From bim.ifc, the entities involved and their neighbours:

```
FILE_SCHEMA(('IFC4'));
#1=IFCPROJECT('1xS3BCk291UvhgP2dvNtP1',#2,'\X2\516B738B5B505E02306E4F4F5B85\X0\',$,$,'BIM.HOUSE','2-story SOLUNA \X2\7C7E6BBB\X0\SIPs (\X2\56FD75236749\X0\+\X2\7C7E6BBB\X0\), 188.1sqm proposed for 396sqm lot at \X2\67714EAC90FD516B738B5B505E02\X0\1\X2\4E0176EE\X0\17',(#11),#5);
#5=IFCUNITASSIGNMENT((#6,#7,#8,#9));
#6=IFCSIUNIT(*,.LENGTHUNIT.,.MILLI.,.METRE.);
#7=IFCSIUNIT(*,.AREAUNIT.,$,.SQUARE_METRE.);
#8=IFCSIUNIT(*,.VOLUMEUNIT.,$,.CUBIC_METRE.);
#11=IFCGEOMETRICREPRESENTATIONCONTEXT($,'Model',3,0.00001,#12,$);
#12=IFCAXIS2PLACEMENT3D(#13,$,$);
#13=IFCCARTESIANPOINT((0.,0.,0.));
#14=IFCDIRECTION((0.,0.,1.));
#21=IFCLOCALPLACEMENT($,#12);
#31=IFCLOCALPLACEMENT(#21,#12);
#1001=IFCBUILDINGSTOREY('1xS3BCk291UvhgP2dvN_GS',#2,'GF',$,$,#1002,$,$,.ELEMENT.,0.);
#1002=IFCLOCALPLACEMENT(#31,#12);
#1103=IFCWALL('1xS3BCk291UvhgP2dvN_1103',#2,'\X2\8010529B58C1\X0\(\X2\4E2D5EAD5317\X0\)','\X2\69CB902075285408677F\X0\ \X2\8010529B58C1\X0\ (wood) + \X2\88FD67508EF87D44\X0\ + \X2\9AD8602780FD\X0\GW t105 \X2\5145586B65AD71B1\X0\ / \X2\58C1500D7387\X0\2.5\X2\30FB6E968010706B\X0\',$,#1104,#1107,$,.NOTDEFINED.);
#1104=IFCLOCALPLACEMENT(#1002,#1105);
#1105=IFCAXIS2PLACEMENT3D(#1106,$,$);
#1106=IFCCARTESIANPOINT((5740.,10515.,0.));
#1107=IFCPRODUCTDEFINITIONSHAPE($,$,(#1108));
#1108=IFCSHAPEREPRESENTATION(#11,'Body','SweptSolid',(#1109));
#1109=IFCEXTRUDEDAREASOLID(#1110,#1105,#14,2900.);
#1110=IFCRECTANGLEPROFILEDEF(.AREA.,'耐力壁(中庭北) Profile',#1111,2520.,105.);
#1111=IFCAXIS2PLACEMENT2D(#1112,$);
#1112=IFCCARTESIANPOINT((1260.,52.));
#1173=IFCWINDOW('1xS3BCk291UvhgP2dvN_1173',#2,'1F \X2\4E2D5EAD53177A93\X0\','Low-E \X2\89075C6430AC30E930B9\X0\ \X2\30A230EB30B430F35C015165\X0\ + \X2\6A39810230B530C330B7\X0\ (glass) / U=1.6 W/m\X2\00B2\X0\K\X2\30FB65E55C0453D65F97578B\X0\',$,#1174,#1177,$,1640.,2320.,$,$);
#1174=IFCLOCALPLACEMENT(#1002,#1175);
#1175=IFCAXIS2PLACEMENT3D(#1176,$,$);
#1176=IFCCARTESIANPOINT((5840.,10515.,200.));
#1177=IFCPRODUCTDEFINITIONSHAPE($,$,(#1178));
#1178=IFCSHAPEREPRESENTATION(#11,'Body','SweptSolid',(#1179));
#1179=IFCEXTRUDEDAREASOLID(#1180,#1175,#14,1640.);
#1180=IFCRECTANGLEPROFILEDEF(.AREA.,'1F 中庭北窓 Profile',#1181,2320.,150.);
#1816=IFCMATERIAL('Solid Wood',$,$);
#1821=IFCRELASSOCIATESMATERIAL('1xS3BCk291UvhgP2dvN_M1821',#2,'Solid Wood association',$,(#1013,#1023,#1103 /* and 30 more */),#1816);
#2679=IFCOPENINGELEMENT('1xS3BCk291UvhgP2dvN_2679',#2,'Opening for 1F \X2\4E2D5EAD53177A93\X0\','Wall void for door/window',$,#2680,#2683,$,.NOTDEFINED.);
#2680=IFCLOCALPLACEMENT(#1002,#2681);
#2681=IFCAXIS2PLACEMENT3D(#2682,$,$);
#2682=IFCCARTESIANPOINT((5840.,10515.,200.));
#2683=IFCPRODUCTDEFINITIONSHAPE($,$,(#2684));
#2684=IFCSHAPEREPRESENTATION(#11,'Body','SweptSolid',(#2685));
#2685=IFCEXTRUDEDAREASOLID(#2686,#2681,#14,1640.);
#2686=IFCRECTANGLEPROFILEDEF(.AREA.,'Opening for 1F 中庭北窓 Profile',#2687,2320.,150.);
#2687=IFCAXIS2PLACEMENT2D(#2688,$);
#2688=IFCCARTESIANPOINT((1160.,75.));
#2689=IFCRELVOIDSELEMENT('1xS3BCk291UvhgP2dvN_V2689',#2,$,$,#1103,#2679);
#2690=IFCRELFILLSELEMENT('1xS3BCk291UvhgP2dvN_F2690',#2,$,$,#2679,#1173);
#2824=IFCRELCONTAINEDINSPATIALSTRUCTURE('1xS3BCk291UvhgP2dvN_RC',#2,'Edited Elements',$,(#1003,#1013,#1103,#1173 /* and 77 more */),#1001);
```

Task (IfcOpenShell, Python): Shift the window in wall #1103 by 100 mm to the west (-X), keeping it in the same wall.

```python
import ifcopenshell
import ifcopenshell.api.geometry
import ifcopenshell.util.placement
import ifcopenshell.util.unit

model = ifcopenshell.open("bim.ifc")
unit_scale = ifcopenshell.util.unit.calculate_unit_scale(model)

window = model.by_guid("1xS3BCk291UvhgP2dvN_1173")
opening = window.FillsVoids[0].RelatingOpeningElement
wall = opening.VoidsElements[0].RelatingBuildingElement

wall_matrix = ifcopenshell.util.placement.get_local_placement(wall.ObjectPlacement)
shift = wall_matrix[:3, 0] * -0.1 / unit_scale
before = ifcopenshell.util.placement.get_local_placement(window.ObjectPlacement)[:3, 3].copy()

# The window is not placed relative to its opening, so move both.
for product in (opening, window):
    matrix = ifcopenshell.util.placement.get_local_placement(product.ObjectPlacement)
    matrix[:3, 3] += shift
    ifcopenshell.api.geometry.edit_object_placement(model, product=product, matrix=matrix, is_si=False)

after = ifcopenshell.util.placement.get_local_placement(window.ObjectPlacement)[:3, 3]
print("window moved by", (after - before).round(3) + 0.0)

model.write("bim_edited.ifc")
```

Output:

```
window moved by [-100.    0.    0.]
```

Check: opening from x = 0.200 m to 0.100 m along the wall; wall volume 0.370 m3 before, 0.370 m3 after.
